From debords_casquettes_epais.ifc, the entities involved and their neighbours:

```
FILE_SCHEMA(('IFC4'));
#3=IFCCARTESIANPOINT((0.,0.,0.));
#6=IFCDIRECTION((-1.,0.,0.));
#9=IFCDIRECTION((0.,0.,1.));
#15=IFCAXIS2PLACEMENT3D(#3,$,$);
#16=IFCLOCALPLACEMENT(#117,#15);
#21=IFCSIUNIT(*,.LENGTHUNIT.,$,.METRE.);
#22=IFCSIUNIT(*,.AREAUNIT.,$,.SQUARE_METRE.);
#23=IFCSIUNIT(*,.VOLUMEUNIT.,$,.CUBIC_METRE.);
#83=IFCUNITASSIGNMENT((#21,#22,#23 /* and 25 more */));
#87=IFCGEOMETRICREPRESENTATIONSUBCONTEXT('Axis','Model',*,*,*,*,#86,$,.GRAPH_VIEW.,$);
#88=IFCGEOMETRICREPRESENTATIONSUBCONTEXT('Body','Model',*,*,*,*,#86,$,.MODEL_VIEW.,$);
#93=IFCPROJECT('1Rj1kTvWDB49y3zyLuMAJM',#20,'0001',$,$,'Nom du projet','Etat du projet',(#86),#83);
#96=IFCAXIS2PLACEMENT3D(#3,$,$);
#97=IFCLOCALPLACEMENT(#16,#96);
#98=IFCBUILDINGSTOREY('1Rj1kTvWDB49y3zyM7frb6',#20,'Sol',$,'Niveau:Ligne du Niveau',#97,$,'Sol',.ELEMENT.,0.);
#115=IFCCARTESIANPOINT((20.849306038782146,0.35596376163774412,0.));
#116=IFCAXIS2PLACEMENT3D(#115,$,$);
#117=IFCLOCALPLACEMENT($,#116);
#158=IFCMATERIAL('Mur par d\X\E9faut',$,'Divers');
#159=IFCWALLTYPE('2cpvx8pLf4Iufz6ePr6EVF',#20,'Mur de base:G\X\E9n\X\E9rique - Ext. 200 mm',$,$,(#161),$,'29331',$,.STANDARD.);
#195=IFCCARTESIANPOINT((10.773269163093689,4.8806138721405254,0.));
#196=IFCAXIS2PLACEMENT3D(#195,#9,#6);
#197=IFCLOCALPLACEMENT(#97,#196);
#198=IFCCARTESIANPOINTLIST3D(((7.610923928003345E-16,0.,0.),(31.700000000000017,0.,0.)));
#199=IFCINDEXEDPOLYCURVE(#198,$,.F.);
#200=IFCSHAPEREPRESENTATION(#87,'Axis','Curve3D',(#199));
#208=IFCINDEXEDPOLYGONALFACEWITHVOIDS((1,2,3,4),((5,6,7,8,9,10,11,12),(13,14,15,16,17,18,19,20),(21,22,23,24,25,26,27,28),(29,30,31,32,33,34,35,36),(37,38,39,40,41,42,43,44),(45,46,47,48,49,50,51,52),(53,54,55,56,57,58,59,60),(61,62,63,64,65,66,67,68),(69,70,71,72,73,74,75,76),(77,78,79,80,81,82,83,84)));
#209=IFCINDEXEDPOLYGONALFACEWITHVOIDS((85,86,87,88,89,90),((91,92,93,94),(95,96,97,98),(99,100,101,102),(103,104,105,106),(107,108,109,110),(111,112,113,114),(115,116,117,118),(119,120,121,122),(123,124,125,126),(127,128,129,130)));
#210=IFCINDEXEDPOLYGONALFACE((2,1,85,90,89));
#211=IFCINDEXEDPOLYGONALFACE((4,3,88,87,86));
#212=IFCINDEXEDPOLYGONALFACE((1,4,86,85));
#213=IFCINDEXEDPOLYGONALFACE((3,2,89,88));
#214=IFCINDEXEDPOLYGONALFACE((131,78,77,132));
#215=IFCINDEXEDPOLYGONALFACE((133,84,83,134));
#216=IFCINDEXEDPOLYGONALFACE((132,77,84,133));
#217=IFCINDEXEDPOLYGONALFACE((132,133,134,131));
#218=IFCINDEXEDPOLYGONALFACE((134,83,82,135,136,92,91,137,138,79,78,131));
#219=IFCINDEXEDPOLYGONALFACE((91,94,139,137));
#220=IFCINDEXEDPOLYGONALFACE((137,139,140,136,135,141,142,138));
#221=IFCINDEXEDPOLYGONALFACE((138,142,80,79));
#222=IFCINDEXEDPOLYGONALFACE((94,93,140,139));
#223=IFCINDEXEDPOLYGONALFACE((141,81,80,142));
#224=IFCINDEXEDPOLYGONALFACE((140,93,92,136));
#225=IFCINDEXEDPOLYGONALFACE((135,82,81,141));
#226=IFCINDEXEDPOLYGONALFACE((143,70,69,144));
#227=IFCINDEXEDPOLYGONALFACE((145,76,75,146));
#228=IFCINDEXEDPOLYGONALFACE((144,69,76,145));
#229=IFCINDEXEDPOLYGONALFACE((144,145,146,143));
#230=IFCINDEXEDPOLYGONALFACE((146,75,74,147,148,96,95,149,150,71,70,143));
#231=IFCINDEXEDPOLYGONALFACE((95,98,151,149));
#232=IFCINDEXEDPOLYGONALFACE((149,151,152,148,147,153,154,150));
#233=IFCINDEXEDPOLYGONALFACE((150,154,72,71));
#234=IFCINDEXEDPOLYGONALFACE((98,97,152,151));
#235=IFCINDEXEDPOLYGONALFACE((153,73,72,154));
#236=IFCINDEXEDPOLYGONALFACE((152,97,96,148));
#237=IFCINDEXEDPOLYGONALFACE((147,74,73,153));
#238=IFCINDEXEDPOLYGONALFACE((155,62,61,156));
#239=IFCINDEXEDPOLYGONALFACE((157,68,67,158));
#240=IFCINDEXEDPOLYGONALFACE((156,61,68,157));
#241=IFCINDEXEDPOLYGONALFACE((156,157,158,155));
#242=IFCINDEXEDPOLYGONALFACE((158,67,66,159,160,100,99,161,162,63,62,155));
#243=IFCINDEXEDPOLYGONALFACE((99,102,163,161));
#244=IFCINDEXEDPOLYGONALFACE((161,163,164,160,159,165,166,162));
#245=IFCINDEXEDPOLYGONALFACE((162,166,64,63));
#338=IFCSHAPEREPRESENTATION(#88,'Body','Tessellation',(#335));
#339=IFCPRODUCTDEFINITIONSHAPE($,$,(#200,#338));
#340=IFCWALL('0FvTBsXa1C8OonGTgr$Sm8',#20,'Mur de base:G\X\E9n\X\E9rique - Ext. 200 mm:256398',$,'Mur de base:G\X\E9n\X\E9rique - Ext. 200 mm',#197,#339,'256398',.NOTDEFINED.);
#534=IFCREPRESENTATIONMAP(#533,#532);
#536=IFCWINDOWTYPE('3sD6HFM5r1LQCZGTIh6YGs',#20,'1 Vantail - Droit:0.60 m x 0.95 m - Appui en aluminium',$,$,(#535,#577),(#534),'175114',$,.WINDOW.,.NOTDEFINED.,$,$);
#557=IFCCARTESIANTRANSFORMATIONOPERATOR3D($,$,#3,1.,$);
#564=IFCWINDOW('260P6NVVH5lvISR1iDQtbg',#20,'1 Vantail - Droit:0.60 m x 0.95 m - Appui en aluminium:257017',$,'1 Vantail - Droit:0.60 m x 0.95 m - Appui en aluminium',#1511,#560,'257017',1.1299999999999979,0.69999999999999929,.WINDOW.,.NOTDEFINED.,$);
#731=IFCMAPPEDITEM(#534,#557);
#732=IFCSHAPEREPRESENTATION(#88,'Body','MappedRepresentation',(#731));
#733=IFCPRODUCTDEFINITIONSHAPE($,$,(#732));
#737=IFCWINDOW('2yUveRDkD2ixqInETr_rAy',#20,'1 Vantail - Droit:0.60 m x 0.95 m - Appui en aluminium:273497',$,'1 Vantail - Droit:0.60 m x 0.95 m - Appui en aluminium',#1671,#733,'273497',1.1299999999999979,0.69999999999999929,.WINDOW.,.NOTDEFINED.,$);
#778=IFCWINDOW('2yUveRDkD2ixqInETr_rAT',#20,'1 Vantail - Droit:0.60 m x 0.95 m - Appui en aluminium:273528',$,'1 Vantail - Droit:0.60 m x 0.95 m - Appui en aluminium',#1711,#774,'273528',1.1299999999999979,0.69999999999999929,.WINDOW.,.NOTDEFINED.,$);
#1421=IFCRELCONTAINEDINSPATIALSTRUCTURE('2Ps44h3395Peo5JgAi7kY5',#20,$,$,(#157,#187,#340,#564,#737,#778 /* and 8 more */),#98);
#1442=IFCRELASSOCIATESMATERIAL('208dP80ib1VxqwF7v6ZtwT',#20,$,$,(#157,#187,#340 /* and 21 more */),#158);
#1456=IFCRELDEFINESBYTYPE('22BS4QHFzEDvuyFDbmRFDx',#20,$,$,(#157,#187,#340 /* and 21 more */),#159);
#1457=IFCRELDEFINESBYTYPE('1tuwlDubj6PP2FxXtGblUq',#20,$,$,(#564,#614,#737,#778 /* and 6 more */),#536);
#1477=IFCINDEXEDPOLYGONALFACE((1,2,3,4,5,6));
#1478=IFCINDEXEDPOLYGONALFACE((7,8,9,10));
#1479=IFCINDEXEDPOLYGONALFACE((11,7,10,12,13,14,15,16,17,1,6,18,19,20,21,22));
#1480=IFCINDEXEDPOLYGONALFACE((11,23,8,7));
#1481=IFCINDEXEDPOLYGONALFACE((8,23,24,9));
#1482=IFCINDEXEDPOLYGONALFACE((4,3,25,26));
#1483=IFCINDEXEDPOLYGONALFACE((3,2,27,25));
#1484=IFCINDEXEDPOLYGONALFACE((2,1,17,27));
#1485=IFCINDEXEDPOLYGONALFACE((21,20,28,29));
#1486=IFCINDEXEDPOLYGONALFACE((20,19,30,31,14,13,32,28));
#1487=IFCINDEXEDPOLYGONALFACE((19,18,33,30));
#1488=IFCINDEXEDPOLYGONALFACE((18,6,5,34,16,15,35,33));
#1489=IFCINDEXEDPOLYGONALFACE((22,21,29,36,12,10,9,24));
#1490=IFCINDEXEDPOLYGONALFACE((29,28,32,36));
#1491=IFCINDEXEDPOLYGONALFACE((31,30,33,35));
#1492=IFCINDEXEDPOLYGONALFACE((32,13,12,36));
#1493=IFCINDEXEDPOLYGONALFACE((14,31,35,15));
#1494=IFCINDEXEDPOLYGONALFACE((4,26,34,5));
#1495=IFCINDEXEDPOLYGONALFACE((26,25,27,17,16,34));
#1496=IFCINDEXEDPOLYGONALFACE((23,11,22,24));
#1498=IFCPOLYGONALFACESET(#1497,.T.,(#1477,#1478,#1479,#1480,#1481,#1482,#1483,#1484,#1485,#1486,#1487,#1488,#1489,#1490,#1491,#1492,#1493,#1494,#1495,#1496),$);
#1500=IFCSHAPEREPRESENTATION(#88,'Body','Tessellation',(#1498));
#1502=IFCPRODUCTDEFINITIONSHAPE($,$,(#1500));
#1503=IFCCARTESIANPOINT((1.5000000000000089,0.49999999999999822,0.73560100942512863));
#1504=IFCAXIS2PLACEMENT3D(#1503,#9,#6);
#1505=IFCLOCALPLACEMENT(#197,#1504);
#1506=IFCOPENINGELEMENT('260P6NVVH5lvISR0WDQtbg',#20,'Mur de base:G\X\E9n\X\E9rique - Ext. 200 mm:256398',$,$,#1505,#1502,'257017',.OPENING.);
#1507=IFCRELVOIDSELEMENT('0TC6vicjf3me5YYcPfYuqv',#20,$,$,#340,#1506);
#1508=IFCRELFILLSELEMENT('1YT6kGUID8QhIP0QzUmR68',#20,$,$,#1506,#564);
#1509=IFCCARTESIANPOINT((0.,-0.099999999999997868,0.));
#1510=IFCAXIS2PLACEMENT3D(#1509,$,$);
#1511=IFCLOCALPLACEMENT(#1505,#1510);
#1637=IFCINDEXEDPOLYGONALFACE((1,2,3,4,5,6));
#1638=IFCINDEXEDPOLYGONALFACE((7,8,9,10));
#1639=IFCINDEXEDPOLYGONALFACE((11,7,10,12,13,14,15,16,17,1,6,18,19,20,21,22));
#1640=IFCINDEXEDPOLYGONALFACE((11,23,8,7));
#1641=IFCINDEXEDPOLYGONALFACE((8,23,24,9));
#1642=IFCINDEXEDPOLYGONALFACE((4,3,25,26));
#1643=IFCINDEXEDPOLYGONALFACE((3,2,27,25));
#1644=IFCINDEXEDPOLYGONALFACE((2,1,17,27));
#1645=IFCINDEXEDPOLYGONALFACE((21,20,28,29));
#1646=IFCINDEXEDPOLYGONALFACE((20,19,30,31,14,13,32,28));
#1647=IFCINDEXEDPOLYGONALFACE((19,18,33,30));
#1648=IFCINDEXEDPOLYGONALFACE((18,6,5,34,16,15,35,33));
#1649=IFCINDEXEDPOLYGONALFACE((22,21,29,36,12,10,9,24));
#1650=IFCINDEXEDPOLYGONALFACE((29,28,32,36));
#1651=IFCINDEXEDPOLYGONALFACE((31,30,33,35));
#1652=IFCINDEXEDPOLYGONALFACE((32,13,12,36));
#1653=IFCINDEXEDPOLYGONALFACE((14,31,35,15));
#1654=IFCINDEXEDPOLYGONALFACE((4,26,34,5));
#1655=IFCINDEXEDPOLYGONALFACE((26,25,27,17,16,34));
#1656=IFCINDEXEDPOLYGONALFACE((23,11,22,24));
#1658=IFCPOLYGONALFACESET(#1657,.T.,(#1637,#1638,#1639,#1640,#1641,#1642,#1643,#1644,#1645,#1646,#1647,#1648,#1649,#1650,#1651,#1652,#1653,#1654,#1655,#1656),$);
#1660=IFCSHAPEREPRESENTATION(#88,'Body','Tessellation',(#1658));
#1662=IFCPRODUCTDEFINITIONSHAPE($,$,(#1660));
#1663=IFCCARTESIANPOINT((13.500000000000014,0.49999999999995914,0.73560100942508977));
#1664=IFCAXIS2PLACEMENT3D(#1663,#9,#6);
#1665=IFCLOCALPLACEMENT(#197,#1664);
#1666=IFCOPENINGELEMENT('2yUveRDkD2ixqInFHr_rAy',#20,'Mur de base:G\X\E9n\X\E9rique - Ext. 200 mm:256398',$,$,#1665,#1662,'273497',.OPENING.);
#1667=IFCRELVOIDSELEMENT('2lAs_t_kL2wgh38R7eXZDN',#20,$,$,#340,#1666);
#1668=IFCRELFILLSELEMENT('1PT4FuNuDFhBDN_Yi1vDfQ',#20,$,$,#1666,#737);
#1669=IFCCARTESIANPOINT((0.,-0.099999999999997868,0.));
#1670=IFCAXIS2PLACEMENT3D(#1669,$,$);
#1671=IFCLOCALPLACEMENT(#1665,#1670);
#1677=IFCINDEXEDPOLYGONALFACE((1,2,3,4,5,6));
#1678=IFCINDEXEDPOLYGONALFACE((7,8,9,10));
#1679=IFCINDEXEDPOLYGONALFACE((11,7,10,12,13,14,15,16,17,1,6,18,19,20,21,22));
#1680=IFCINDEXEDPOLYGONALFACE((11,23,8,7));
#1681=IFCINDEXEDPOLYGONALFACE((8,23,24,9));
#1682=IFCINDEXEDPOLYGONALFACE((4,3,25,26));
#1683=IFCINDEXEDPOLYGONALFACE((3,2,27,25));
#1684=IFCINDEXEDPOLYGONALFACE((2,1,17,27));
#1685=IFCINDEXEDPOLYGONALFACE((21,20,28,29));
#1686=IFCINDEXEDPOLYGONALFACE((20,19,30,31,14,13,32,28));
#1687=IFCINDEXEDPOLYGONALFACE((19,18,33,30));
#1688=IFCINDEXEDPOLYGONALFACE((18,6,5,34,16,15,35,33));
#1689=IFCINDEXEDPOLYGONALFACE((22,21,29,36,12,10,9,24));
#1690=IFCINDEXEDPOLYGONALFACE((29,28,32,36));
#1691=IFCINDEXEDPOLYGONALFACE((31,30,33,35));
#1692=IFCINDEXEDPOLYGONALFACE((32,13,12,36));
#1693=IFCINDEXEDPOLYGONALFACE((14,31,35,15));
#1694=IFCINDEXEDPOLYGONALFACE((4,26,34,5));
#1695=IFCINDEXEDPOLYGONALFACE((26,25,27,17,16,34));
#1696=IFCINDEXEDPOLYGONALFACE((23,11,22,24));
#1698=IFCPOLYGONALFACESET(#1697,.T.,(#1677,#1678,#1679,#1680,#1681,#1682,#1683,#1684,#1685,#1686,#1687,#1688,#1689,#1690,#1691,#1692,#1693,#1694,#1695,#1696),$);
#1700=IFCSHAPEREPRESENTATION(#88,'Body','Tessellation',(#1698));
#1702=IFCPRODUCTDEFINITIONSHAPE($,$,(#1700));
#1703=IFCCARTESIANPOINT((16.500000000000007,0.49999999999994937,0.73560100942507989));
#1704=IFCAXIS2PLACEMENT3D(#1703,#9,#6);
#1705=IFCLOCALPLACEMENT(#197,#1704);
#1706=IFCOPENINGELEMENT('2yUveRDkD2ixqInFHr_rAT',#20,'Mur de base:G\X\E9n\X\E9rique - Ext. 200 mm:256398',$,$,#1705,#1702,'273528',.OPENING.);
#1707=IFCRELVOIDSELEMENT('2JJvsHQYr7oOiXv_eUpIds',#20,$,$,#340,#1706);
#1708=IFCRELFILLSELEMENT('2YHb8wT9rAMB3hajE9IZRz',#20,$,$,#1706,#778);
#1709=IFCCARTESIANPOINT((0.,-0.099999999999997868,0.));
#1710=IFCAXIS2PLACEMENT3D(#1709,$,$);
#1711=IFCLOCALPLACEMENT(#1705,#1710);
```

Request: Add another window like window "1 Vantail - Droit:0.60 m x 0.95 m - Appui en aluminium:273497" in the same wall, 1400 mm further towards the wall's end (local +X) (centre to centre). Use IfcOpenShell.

```python
import ifcopenshell
import ifcopenshell.api.feature
import ifcopenshell.api.geometry
import ifcopenshell.api.root
import ifcopenshell.geom
import ifcopenshell.util.element
import ifcopenshell.util.placement
import ifcopenshell.util.shape

model = ifcopenshell.open("debords_casquettes_epais.ifc")
settings = ifcopenshell.geom.settings()


def volume(element):
    """Net volume in cubic metres, openings subtracted."""
    shape = ifcopenshell.geom.create_shape(settings, element)
    return ifcopenshell.util.shape.get_volume(shape.geometry)


def reuse_history(source, copy):
    """copy_class also copies each property set's owner history, people and application; keep the originals."""
    for rel in copy.IsDefinedBy:
        if rel.is_a("IfcRelDefinesByProperties") and (history := rel.RelatingPropertyDefinition.OwnerHistory):
            rel.RelatingPropertyDefinition.OwnerHistory = source.OwnerHistory
            ifcopenshell.util.element.remove_deep2(model, history)


window = model.by_guid("2yUveRDkD2ixqInETr_rAy")
opening = window.FillsVoids[0].RelatingOpeningElement
wall = opening.VoidsElements[0].RelatingBuildingElement
before = volume(wall)
shift = ifcopenshell.util.placement.get_local_placement(wall.ObjectPlacement)[:3, 0] * 1.4

# copy_class copies the void relationship, type, container and properties, but no geometry.
new_opening = ifcopenshell.api.root.copy_class(model, product=opening)
new_opening.Representation = ifcopenshell.util.element.copy_deep(
    model, opening.Representation, exclude=["IfcGeometricRepresentationContext", "IfcRepresentationMap"]
)
new_opening.Name = "Mur de base:Générique - Ext. 200 mm"
new_opening.Tag = None
new_window = ifcopenshell.api.root.copy_class(model, product=window)
new_window.Representation = ifcopenshell.util.element.copy_deep(
    model, window.Representation, exclude=["IfcGeometricRepresentationContext", "IfcRepresentationMap"]
)
new_window.Name = "1 Vantail - Droit:0.60 m x 0.95 m - Appui en aluminium"
new_window.Tag = None
reuse_history(window, new_window)
ifcopenshell.api.feature.add_filling(model, opening=new_opening, element=new_window)

for old, new in ((opening, new_opening), (window, new_window)):
    matrix = ifcopenshell.util.placement.get_local_placement(old.ObjectPlacement)
    matrix[:3, 3] += shift
    ifcopenshell.api.geometry.edit_object_placement(model, product=new, matrix=matrix, is_si=False)

after = volume(wall)

print(f"wall volume {before:.3f} -> {after:.3f} m3")

model.write("debords_casquettes_epais_updated.ifc")
```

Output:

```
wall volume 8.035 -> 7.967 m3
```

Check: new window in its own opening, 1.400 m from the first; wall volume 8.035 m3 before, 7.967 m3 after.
